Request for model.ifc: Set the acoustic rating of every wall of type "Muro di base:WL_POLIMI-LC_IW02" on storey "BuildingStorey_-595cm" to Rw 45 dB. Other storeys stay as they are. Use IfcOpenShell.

First a look at what the model holds.

```python
import ifcopenshell
import ifcopenshell.util.element

model = ifcopenshell.open("model.ifc")
print(model.schema)
storey = next(s for s in model.by_type("IfcBuildingStorey") if s.Name == "BuildingStorey_-595cm")
walls = [e for e in ifcopenshell.util.element.get_decomposition(storey) if e.is_a("IfcWall")]
seen = {}
for e in walls:
    element_type = ifcopenshell.util.element.get_type(e)
    key = (element_type.Name if element_type != e and element_type else None, ifcopenshell.util.element.get_pset(e, "Pset_WallCommon", "AcousticRating"))
    seen[key] = seen.get(key, 0) + 1
for (name, value), count in sorted(seen.items(), key=str):
    print(count, "x", name, "|", value)
```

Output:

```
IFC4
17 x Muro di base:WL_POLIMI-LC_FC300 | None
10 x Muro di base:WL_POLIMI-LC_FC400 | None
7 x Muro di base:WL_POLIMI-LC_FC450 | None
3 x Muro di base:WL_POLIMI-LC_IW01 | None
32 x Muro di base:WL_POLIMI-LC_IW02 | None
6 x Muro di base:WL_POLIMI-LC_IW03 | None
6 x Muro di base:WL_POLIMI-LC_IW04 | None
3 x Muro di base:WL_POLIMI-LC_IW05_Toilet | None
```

```python
import ifcopenshell
import ifcopenshell.api.pset
import ifcopenshell.util.element

model = ifcopenshell.open("model.ifc")

storey = next(s for s in model.by_type("IfcBuildingStorey") if s.Name == "BuildingStorey_-595cm")
walls = [e for e in ifcopenshell.util.element.get_decomposition(storey) if e.is_a("IfcWall")]

count = 0
for e in walls:
    element_type = ifcopenshell.util.element.get_type(e)
    if element_type in (None, e) or element_type.Name != "Muro di base:WL_POLIMI-LC_IW02":
        continue
    # add_pset returns the element's existing set when there is one.
    pset = ifcopenshell.api.pset.add_pset(model, product=e, name="Pset_WallCommon")
    ifcopenshell.api.pset.edit_pset(model, pset=pset, properties={"AcousticRating": "Rw 45 dB"})
    count += 1

print(count, "walls updated")

model.write("model_v2.ifc")
```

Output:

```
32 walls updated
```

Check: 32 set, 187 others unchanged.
